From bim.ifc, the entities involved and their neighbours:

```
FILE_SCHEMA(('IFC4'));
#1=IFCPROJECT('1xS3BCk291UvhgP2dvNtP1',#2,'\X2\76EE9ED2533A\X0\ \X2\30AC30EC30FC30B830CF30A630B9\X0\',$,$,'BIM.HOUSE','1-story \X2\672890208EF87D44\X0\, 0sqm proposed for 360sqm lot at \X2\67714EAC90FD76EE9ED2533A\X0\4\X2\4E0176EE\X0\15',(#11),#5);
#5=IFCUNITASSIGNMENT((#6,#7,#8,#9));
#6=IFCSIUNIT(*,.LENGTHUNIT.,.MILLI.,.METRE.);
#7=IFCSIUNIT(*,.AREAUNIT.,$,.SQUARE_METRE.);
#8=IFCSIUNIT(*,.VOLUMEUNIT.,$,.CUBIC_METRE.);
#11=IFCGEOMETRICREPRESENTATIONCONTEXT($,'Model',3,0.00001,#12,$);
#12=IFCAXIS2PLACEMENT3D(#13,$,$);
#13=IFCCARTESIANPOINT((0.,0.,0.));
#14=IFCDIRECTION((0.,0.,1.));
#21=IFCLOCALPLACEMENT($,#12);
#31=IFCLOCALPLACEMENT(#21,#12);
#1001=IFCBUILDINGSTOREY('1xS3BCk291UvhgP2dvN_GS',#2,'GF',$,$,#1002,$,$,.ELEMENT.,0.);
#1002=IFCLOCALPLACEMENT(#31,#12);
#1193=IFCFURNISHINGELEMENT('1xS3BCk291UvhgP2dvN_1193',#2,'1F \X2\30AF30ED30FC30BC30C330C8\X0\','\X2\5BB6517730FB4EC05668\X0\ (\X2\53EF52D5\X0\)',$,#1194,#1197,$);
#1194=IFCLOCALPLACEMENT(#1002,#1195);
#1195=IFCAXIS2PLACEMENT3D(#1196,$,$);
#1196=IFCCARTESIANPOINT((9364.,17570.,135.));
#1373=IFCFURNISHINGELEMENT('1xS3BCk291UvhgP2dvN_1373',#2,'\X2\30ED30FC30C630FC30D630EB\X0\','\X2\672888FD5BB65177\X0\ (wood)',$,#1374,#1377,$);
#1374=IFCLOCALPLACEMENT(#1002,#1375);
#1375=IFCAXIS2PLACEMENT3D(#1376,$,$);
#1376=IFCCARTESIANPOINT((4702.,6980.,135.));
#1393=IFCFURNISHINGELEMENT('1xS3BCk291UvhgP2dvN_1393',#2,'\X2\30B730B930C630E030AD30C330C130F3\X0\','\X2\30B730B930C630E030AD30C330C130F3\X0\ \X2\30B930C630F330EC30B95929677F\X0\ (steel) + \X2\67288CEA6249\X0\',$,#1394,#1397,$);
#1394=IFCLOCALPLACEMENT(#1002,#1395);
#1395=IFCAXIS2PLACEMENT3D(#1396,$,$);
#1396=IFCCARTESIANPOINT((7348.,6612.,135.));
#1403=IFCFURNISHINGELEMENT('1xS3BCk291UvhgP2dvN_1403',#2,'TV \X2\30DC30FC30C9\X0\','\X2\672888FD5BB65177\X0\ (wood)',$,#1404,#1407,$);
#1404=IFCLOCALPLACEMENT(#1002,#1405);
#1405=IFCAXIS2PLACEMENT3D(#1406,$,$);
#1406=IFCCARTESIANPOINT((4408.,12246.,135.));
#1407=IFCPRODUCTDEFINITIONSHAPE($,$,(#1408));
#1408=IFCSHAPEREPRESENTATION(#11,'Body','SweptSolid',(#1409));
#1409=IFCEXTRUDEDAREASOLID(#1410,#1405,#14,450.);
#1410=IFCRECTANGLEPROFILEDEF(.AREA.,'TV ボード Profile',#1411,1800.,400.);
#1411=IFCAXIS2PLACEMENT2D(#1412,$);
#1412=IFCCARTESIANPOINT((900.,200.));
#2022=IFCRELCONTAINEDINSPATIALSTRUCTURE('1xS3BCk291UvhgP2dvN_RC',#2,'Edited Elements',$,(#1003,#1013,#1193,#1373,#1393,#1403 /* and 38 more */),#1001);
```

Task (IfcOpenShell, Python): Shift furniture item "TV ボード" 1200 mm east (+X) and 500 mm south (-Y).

```python
import ifcopenshell
import ifcopenshell.api.geometry
import ifcopenshell.util.placement
import ifcopenshell.util.unit

model = ifcopenshell.open("bim.ifc")
unit_scale = ifcopenshell.util.unit.calculate_unit_scale(model)

item = model.by_guid("1xS3BCk291UvhgP2dvN_1403")
matrix = ifcopenshell.util.placement.get_local_placement(item.ObjectPlacement)
matrix[0, 3] += 1.2 / unit_scale
matrix[1, 3] -= 0.5 / unit_scale
ifcopenshell.api.geometry.edit_object_placement(model, product=item, matrix=matrix, is_si=False)

print(ifcopenshell.util.placement.get_local_placement(item.ObjectPlacement).round(3) + 0.0)

model.write("bim_rev.ifc")
```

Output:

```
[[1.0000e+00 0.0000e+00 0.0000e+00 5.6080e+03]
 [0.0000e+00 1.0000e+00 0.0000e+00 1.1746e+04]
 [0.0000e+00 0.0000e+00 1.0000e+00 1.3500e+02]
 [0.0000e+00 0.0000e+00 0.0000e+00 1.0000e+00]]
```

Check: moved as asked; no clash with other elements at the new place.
